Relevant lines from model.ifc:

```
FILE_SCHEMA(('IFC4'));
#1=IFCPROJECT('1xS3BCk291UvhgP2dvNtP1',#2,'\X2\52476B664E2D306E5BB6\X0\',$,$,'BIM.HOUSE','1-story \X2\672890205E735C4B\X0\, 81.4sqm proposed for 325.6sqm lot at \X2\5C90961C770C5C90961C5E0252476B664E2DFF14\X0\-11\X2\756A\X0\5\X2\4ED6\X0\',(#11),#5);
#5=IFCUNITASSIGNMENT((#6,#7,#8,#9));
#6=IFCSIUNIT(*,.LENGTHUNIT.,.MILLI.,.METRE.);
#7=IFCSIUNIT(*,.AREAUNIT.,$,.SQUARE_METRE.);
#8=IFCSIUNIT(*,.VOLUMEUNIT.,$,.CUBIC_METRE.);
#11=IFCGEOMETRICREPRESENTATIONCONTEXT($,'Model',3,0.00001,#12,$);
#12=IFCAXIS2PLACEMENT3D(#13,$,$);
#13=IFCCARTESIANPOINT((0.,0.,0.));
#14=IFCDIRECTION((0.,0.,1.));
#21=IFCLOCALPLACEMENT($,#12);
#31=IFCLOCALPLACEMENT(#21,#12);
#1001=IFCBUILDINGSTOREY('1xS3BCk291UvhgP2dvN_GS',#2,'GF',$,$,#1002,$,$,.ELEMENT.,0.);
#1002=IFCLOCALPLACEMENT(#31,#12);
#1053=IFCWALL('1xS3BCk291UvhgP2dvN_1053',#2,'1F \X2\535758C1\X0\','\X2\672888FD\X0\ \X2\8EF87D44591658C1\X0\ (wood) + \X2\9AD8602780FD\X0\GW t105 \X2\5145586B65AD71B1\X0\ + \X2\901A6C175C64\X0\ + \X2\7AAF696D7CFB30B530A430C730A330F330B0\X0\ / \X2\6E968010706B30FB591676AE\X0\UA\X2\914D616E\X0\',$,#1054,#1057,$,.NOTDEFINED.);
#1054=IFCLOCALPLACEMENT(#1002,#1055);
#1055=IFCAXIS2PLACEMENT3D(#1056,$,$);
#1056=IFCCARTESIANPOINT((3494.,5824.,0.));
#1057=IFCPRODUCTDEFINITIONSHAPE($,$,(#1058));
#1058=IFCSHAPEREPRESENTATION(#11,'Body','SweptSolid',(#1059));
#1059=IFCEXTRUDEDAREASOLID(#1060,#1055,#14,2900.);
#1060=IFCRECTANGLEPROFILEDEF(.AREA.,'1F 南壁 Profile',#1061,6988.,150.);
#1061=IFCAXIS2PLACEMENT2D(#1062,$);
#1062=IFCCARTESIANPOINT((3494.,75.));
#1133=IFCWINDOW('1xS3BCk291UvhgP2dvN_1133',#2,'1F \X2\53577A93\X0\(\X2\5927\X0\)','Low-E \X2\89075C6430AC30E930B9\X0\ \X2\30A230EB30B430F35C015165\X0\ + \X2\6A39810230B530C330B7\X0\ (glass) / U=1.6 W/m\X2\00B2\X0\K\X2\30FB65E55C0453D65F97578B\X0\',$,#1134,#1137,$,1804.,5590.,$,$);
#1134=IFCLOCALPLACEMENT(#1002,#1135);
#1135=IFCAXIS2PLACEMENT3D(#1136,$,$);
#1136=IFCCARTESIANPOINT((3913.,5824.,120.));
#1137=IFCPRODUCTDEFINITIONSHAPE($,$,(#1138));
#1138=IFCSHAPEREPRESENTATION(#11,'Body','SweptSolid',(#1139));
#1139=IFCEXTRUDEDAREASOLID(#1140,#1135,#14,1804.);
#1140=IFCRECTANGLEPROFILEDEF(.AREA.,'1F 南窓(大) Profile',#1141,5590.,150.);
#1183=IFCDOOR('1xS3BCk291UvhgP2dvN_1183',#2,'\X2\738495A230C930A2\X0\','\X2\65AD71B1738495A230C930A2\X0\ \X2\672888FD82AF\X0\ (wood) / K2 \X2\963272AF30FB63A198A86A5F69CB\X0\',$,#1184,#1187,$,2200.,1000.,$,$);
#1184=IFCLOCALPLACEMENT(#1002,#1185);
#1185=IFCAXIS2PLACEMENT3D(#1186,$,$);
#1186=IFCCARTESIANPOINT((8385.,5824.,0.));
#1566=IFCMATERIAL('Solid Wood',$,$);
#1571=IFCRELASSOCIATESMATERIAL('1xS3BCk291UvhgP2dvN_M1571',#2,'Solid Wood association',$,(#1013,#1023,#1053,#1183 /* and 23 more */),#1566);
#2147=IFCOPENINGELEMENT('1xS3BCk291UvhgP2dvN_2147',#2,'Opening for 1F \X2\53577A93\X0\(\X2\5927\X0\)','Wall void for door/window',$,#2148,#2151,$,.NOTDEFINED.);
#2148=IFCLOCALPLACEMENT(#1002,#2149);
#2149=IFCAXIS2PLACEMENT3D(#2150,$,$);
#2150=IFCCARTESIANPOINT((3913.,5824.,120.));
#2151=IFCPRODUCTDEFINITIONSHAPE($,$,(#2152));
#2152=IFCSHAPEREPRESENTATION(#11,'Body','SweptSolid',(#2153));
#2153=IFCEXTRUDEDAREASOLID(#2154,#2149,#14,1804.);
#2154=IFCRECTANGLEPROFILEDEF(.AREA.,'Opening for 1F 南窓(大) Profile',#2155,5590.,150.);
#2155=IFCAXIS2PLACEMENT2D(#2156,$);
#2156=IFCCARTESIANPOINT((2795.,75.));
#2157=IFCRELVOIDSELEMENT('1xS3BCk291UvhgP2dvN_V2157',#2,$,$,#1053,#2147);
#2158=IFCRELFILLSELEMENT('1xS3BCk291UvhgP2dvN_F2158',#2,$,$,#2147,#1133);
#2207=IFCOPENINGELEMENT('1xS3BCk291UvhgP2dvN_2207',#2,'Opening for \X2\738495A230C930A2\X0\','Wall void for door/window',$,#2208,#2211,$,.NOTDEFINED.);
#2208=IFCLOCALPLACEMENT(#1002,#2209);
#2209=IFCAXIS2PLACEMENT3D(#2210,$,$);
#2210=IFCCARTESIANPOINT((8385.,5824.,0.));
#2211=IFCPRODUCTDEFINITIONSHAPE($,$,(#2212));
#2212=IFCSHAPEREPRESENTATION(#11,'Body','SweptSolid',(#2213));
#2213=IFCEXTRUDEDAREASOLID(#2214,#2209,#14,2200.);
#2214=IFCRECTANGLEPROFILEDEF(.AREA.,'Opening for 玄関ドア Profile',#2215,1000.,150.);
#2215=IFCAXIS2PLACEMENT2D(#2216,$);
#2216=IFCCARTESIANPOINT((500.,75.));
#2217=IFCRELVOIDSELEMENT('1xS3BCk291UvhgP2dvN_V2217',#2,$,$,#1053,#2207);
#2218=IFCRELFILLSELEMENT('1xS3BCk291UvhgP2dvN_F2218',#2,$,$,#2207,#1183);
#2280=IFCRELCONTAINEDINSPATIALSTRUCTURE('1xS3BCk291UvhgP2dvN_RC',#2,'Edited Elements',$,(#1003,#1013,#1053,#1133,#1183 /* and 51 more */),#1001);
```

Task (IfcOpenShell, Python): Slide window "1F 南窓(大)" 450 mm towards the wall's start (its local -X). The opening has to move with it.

```python
import ifcopenshell
import ifcopenshell.api.geometry
import ifcopenshell.util.placement

model = ifcopenshell.open("model.ifc")

window = model.by_guid("1xS3BCk291UvhgP2dvN_1133")
opening = window.FillsVoids[0].RelatingOpeningElement
wall = opening.VoidsElements[0].RelatingBuildingElement

wall_matrix = ifcopenshell.util.placement.get_local_placement(wall.ObjectPlacement)
shift = wall_matrix[:3, 0] * -450.0
before = ifcopenshell.util.placement.get_local_placement(window.ObjectPlacement)[:3, 3].copy()

# The window is not placed relative to its opening, so move both.
for product in (opening, window):
    matrix = ifcopenshell.util.placement.get_local_placement(product.ObjectPlacement)
    matrix[:3, 3] += shift
    ifcopenshell.api.geometry.edit_object_placement(model, product=product, matrix=matrix, is_si=False)

after = ifcopenshell.util.placement.get_local_placement(window.ObjectPlacement)[:3, 3]
print("window moved by", (after - before).round(3) + 0.0)

model.write("model_rev.ifc")
```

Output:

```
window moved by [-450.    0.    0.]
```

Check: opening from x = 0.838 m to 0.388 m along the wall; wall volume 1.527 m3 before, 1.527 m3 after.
